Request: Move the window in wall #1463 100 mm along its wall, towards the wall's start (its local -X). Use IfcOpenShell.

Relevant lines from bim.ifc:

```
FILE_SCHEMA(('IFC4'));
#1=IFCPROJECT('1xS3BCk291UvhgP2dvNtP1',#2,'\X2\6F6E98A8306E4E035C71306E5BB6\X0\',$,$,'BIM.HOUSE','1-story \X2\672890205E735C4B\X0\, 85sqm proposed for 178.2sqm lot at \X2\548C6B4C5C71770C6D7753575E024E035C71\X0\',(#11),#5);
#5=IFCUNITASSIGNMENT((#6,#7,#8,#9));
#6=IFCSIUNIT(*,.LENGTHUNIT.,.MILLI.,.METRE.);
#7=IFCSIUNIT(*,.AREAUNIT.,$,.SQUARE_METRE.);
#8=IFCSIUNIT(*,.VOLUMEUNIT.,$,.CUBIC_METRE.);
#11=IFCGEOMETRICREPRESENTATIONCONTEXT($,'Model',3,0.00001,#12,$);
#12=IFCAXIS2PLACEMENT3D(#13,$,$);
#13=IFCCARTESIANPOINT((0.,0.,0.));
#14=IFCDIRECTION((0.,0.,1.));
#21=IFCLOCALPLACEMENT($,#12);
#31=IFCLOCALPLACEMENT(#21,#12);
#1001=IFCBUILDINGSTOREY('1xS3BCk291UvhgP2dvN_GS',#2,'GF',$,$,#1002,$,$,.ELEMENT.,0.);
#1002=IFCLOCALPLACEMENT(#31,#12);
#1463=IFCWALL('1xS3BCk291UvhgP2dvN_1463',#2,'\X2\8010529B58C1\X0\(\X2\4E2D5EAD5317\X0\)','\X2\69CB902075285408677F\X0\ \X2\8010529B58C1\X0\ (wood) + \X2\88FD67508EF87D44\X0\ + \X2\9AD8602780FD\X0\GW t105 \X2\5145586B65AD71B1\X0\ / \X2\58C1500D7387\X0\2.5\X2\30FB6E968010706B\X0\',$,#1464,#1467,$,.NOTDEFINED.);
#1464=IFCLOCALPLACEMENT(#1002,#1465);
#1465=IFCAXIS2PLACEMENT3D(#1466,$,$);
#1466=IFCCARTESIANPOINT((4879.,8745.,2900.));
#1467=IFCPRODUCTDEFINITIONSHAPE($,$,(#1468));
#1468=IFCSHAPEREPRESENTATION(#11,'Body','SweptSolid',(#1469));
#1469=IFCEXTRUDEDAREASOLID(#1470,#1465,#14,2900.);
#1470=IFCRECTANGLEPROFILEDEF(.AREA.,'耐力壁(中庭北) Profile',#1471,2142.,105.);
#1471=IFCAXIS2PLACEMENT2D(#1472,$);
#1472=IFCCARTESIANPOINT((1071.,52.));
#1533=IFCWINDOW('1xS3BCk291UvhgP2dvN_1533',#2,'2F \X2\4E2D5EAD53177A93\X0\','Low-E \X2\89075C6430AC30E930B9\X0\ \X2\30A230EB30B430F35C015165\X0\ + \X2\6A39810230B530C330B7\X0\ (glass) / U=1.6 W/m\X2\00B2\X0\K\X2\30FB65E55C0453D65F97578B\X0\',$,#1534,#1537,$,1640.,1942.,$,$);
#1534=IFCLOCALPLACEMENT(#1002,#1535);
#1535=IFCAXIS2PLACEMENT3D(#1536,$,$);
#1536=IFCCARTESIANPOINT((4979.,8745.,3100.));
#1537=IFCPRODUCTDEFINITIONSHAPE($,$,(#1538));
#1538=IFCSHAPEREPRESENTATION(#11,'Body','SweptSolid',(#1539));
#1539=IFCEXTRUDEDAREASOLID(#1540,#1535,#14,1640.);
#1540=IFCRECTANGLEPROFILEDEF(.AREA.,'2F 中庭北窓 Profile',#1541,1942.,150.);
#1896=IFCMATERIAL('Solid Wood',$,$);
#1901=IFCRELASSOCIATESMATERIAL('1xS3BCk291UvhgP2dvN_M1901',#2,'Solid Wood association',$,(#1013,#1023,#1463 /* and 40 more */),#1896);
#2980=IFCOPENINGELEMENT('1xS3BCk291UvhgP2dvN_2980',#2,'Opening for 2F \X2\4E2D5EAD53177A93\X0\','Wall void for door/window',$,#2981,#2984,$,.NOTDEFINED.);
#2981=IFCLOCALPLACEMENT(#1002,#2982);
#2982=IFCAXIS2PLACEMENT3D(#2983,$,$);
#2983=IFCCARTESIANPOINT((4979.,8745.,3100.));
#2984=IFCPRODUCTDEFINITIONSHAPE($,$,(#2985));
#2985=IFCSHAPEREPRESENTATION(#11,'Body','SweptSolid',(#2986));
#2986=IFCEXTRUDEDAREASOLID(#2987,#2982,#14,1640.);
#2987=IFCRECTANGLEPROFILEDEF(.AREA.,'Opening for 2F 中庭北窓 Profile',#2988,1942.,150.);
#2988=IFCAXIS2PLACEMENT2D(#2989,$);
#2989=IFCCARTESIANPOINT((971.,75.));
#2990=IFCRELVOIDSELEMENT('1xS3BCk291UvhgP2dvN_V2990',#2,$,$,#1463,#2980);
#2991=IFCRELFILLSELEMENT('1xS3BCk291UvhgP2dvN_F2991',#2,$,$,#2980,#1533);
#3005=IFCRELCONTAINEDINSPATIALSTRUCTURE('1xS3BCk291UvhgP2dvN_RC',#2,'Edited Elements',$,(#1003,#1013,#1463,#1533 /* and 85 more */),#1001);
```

```python
import ifcopenshell
import ifcopenshell.api.geometry
import ifcopenshell.util.placement
import ifcopenshell.util.unit

model = ifcopenshell.open("bim.ifc")
unit_scale = ifcopenshell.util.unit.calculate_unit_scale(model)

window = model.by_guid("1xS3BCk291UvhgP2dvN_1533")
opening = window.FillsVoids[0].RelatingOpeningElement
wall = opening.VoidsElements[0].RelatingBuildingElement

wall_matrix = ifcopenshell.util.placement.get_local_placement(wall.ObjectPlacement)
shift = wall_matrix[:3, 0] * -0.1 / unit_scale
before = ifcopenshell.util.placement.get_local_placement(window.ObjectPlacement)[:3, 3].copy()

# The window is not placed relative to its opening, so move both.
for product in (opening, window):
    matrix = ifcopenshell.util.placement.get_local_placement(product.ObjectPlacement)
    matrix[:3, 3] += shift
    ifcopenshell.api.geometry.edit_object_placement(model, product=product, matrix=matrix, is_si=False)

after = ifcopenshell.util.placement.get_local_placement(window.ObjectPlacement)[:3, 3]
print("window moved by", (after - before).round(3) + 0.0)

model.write("bim_rev.ifc")
```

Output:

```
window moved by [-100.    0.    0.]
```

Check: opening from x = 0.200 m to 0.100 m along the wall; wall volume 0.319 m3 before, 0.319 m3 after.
